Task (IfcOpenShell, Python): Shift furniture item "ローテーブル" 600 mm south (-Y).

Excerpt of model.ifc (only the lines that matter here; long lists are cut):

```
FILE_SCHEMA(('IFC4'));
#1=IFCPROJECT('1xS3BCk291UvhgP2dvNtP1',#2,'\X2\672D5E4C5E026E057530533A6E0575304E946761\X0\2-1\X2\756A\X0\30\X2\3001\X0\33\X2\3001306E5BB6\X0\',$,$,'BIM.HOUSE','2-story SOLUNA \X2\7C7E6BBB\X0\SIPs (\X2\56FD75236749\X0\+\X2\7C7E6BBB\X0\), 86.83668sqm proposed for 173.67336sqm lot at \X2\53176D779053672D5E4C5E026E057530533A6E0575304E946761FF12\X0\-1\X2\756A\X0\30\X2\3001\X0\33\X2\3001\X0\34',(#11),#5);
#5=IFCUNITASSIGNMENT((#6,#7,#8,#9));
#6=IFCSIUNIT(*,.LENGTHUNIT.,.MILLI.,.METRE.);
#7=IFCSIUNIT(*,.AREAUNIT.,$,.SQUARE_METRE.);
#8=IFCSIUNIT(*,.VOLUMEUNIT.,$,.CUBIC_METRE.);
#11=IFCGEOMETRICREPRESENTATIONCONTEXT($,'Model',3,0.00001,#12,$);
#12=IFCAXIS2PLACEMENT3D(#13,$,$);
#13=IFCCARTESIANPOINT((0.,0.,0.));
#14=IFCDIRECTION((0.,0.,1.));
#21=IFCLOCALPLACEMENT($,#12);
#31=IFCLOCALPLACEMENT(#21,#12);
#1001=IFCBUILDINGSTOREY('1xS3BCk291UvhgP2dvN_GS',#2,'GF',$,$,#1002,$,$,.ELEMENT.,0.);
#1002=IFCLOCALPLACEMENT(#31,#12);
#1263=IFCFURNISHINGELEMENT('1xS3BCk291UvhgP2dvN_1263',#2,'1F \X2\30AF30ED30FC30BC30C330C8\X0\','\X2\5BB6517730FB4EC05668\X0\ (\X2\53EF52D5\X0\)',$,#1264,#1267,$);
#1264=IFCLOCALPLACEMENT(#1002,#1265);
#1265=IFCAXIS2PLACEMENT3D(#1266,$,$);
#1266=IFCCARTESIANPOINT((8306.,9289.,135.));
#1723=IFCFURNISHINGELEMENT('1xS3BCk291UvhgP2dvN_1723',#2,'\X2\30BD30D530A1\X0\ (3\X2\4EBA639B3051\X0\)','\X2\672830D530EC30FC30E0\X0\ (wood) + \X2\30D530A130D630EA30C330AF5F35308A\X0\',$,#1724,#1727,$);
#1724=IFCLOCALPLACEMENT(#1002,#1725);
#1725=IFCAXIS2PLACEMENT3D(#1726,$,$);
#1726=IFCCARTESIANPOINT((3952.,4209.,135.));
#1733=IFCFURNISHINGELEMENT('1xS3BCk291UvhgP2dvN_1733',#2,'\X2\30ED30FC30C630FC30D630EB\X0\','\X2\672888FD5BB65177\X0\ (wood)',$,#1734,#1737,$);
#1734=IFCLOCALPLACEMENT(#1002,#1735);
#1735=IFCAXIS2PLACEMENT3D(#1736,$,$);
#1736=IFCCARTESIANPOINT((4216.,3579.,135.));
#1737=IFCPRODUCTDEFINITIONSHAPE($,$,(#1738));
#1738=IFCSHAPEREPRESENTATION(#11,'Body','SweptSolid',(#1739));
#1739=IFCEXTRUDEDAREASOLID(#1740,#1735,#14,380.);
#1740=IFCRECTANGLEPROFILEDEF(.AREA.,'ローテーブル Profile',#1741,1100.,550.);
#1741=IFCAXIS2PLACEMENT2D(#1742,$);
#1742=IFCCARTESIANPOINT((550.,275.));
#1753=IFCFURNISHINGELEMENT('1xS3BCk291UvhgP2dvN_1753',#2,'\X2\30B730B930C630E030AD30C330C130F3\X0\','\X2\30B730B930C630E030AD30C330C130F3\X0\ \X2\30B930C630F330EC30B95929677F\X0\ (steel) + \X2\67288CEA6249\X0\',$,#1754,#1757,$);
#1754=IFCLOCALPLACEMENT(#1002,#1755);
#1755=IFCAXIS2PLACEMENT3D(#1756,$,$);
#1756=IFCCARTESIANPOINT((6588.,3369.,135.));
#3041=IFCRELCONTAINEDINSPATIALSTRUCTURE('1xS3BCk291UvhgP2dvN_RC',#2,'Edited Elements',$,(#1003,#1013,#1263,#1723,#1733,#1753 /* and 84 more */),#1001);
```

```python
import ifcopenshell
import ifcopenshell.api.geometry
import ifcopenshell.util.placement
import ifcopenshell.util.unit

model = ifcopenshell.open("model.ifc")
unit_scale = ifcopenshell.util.unit.calculate_unit_scale(model)

item = model.by_guid("1xS3BCk291UvhgP2dvN_1733")
matrix = ifcopenshell.util.placement.get_local_placement(item.ObjectPlacement)
matrix[1, 3] -= 0.6 / unit_scale
ifcopenshell.api.geometry.edit_object_placement(model, product=item, matrix=matrix, is_si=False)

print(ifcopenshell.util.placement.get_local_placement(item.ObjectPlacement).round(3) + 0.0)

model.write("model_rev.ifc")
```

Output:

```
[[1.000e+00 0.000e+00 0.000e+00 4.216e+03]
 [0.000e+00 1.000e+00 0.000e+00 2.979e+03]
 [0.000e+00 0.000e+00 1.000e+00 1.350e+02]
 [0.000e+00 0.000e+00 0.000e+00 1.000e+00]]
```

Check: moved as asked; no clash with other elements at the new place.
